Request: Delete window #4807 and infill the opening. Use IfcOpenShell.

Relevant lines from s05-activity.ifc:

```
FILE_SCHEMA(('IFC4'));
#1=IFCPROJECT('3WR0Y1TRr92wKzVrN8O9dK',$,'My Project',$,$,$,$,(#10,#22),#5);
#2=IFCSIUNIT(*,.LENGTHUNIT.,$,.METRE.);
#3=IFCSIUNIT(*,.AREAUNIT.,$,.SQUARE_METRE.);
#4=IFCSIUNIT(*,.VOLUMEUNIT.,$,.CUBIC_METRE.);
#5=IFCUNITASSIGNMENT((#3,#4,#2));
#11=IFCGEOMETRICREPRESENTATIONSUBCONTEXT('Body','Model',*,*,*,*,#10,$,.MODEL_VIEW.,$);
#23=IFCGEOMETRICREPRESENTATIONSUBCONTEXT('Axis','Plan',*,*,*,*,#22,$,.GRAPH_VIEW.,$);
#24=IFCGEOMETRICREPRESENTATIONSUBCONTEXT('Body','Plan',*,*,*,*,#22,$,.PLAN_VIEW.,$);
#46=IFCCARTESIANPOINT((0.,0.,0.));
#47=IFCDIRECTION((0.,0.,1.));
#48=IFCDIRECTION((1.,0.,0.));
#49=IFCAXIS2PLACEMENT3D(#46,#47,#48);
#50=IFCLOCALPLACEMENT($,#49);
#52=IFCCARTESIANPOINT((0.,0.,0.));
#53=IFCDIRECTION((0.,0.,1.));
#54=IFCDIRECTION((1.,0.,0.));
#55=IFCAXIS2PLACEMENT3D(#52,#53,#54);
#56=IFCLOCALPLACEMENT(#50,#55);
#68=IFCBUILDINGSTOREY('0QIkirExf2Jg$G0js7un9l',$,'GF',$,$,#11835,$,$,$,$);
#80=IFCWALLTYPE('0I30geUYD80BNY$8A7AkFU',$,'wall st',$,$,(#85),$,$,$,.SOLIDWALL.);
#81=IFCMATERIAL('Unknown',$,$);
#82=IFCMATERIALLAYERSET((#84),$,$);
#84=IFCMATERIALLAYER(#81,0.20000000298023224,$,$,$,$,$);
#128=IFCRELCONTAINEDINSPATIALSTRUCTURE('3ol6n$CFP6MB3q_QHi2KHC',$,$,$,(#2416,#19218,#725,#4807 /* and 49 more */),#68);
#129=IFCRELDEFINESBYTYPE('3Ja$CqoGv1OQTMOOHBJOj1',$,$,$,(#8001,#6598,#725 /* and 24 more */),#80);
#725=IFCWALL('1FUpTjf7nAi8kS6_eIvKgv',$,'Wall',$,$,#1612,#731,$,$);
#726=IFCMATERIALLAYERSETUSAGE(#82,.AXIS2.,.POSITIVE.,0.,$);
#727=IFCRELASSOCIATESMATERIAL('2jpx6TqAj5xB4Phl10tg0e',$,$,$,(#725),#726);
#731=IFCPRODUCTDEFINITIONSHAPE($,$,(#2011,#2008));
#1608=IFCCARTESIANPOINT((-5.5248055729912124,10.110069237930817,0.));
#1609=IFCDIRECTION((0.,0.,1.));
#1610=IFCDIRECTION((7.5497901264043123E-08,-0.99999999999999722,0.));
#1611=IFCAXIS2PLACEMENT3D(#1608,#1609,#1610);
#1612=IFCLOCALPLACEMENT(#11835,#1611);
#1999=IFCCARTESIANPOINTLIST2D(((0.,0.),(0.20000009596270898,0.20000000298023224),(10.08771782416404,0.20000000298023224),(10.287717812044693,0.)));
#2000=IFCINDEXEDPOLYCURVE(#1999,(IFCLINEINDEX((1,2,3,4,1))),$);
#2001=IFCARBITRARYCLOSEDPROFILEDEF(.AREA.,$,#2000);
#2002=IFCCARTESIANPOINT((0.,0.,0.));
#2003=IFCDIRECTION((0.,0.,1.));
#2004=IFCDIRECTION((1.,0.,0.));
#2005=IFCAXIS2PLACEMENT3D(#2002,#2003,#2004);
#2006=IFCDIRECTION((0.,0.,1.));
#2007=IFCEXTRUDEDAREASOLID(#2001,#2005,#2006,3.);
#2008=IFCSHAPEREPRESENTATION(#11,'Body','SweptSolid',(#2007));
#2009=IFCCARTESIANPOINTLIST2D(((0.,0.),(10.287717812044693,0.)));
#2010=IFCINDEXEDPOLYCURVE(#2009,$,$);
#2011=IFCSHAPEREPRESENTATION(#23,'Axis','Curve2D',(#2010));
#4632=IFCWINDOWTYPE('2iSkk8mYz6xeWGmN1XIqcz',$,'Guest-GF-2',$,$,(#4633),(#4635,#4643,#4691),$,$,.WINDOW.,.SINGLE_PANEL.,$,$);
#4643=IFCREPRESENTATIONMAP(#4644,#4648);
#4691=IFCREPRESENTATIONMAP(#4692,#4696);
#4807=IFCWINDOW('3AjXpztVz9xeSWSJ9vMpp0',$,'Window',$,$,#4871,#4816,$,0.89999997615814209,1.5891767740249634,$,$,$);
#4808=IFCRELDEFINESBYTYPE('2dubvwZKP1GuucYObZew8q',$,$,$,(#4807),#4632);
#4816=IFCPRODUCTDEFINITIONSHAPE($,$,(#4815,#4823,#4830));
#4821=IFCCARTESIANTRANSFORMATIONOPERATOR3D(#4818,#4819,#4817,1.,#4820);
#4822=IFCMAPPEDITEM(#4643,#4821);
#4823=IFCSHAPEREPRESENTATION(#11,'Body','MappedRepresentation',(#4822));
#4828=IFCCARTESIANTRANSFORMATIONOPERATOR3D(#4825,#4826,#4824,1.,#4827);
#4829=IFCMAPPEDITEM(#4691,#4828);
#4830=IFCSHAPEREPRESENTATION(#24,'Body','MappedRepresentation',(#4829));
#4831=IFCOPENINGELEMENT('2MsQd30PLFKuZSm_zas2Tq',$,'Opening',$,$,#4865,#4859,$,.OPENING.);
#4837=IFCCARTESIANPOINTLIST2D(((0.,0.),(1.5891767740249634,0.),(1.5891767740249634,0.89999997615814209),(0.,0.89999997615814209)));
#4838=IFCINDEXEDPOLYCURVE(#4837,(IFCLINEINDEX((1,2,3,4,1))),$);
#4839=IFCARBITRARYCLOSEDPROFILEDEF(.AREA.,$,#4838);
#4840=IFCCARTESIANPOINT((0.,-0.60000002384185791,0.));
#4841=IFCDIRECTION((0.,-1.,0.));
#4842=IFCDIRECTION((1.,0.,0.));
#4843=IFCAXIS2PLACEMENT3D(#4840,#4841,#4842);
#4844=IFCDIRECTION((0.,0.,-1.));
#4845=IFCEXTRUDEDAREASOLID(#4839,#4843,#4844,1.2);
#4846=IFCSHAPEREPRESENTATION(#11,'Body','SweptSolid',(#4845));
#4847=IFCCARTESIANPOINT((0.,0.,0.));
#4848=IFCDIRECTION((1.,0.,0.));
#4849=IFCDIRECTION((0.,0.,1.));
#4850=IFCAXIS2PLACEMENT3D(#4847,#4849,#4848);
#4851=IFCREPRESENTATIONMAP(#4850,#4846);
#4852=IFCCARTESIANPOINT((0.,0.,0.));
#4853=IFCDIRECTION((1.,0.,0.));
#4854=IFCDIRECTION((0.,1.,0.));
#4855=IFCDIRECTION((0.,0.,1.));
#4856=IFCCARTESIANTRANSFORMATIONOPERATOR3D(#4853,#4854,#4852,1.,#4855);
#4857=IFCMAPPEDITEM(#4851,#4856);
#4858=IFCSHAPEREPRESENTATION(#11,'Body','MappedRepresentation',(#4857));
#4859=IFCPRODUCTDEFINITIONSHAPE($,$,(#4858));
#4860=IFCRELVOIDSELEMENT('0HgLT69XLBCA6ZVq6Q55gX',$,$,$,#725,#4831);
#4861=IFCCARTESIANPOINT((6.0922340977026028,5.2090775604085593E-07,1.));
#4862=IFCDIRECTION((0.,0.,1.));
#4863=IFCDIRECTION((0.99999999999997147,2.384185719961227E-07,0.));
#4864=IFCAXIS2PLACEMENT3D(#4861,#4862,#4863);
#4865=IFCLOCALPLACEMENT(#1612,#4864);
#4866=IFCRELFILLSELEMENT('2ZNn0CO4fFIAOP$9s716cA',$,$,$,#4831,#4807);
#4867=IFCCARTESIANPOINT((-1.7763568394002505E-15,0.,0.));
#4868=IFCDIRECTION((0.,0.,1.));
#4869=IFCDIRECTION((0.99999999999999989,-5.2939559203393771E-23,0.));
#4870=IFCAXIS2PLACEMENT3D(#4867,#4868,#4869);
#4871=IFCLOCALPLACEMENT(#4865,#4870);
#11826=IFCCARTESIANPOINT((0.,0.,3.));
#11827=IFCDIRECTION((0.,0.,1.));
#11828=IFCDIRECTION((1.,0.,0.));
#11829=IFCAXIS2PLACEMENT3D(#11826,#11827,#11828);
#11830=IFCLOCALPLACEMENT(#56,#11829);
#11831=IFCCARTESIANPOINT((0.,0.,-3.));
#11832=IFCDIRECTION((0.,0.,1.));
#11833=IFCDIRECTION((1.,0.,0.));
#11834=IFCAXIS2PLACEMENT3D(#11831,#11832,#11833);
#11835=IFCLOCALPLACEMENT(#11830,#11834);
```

```python
import ifcopenshell
import ifcopenshell.api.feature
import ifcopenshell.api.root
import ifcopenshell.geom
import ifcopenshell.util.shape

model = ifcopenshell.open("s05-activity.ifc")
settings = ifcopenshell.geom.settings()


def volume(element):
    """Net volume in cubic metres, openings subtracted."""
    shape = ifcopenshell.geom.create_shape(settings, element)
    return ifcopenshell.util.shape.get_volume(shape.geometry)


window = model.by_guid("3AjXpztVz9xeSWSJ9vMpp0")
opening = window.FillsVoids[0].RelatingOpeningElement
wall = opening.VoidsElements[0].RelatingBuildingElement
before = volume(wall)

ifcopenshell.api.root.remove_product(model, product=window)
ifcopenshell.api.feature.remove_feature(model, feature=opening)

after = volume(wall)

print(f"wall volume {before:.3f} -> {after:.3f} m3")

model.write("s05-activity-out.ifc")
```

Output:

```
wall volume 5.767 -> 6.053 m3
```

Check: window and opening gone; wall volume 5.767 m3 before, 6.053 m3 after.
